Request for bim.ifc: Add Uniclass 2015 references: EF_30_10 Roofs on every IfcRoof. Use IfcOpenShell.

First a look at what the model holds.

```python
import ifcopenshell

model = ifcopenshell.open("bim.ifc")
print(model.schema)
print("classifications:", [c.Name for c in model.by_type("IfcClassification")])
for ifc_class in ("IfcDoor", "IfcRoof", "IfcStair", "IfcWall", "IfcWindow"):
    print(ifc_class, len(model.by_type(ifc_class)))
```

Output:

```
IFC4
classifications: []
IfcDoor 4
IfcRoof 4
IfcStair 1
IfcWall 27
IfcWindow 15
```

```python
import ifcopenshell
import ifcopenshell.api.classification

model = ifcopenshell.open("bim.ifc")

system = ifcopenshell.api.classification.add_classification(model, classification="Uniclass 2015")

codes = {
    "IfcRoof": ("EF_30_10", "Roofs"),
}
for ifc_class, (code, name) in codes.items():
    products = model.by_type(ifc_class)
    ifcopenshell.api.classification.add_reference(
        model, products=products, classification=system, identification=code, name=name
    )
    print(code, len(products))

model.write("bim_v2.ifc")
```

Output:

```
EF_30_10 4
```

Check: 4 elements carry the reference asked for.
